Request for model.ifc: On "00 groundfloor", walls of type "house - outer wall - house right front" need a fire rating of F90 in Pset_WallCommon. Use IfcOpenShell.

First a look at what the model holds.

```python
import ifcopenshell
import ifcopenshell.util.element

model = ifcopenshell.open("model.ifc")
print(model.schema)
storey = next(s for s in model.by_type("IfcBuildingStorey") if s.Name == "00 groundfloor")
walls = [e for e in ifcopenshell.util.element.get_decomposition(storey) if e.is_a("IfcWall")]
seen = {}
for e in walls:
    element_type = ifcopenshell.util.element.get_type(e)
    key = (element_type.Name if element_type != e and element_type else None, ifcopenshell.util.element.get_pset(e, "Pset_WallCommon", "FireRating"))
    seen[key] = seen.get(key, 0) + 1
for (name, value), count in sorted(seen.items(), key=str):
    print(count, "x", name, "|", value)
```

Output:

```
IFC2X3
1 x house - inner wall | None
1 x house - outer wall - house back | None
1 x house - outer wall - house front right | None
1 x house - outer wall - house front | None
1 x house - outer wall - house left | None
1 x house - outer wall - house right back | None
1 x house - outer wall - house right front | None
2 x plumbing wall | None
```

```python
import ifcopenshell
import ifcopenshell.api.pset
import ifcopenshell.util.element

model = ifcopenshell.open("model.ifc")

storey = next(s for s in model.by_type("IfcBuildingStorey") if s.Name == "00 groundfloor")
walls = [e for e in ifcopenshell.util.element.get_decomposition(storey) if e.is_a("IfcWall")]

count = 0
for e in walls:
    element_type = ifcopenshell.util.element.get_type(e)
    if element_type in (None, e) or element_type.Name != "house - outer wall - house right front":
        continue
    # add_pset returns the element's existing set when there is one.
    pset = ifcopenshell.api.pset.add_pset(model, product=e, name="Pset_WallCommon")
    ifcopenshell.api.pset.edit_pset(model, pset=pset, properties={"FireRating": "F90"})
    count += 1

print(count, "walls updated")

model.write("model-out.ifc")
```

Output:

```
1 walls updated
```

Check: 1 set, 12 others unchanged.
